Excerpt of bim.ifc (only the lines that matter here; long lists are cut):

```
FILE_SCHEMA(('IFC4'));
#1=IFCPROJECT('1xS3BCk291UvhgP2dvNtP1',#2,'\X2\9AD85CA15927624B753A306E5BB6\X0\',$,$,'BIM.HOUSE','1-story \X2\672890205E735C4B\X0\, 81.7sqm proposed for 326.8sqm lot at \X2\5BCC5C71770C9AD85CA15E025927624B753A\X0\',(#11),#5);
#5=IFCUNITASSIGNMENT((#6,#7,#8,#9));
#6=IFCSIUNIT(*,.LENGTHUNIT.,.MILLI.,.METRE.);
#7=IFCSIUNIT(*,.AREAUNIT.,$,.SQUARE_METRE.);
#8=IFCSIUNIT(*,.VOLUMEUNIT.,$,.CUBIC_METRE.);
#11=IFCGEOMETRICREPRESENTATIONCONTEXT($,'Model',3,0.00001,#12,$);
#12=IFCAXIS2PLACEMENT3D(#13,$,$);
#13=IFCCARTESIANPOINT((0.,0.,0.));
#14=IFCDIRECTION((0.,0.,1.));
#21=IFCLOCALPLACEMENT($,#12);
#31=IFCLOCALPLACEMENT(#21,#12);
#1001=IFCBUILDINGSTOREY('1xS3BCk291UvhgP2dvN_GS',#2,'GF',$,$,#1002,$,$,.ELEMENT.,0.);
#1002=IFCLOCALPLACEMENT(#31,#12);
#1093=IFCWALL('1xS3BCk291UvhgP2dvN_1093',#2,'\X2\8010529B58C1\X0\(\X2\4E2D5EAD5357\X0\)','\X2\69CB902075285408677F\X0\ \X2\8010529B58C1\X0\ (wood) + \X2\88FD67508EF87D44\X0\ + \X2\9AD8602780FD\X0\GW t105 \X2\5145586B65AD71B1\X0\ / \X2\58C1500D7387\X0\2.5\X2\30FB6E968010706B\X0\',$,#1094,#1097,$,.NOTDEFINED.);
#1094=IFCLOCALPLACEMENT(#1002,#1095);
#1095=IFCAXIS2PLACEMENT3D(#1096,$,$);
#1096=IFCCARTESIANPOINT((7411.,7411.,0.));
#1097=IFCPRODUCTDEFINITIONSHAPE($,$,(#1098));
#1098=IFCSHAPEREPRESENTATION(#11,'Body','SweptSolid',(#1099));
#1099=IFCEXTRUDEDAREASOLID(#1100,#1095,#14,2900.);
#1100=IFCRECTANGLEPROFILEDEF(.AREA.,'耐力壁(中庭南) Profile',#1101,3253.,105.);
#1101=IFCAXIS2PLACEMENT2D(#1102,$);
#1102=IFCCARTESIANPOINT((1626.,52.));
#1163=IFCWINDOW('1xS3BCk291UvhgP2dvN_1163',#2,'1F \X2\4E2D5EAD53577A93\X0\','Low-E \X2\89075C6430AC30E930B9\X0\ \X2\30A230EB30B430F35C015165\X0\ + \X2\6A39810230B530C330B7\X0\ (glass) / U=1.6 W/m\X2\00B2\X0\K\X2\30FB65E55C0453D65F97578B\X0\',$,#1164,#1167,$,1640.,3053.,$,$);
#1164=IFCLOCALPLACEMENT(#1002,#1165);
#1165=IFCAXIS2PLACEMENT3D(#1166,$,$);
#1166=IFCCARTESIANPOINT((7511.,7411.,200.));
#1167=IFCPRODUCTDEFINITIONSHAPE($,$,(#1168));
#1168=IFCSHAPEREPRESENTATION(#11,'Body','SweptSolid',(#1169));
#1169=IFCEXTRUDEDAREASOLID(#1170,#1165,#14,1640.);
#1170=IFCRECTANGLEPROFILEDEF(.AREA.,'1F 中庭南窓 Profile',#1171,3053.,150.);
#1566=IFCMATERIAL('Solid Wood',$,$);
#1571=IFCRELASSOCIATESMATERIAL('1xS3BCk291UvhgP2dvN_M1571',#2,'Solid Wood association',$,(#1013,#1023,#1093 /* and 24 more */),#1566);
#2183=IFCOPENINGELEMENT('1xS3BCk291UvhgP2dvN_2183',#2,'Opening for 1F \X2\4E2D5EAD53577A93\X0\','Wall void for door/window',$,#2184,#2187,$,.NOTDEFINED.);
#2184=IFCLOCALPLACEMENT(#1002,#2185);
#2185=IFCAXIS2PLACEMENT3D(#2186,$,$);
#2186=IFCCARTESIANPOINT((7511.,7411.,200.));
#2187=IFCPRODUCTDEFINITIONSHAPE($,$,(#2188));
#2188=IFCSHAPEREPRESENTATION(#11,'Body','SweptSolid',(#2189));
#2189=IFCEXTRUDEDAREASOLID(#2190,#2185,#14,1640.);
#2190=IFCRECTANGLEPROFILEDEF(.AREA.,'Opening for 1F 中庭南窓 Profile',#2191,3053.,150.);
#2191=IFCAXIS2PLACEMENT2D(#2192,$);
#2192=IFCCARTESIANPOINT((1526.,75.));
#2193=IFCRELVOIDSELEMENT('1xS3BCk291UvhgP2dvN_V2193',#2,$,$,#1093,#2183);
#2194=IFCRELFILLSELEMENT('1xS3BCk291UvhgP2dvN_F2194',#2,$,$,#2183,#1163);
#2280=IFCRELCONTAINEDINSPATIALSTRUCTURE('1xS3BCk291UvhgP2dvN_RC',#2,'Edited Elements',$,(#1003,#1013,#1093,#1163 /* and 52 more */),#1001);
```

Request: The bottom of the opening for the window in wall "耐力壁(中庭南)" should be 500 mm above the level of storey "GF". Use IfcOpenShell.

```python
import numpy as np
import ifcopenshell
import ifcopenshell.api.geometry
import ifcopenshell.geom
import ifcopenshell.util.element
import ifcopenshell.util.placement
import ifcopenshell.util.shape
import ifcopenshell.util.unit

model = ifcopenshell.open("bim.ifc")
unit_scale = ifcopenshell.util.unit.calculate_unit_scale(model)

window = model.by_guid("1xS3BCk291UvhgP2dvN_1163")
opening = window.FillsVoids[0].RelatingOpeningElement
storey = ifcopenshell.util.element.get_container(window, ifc_class="IfcBuildingStorey")
level = ifcopenshell.util.placement.get_local_placement(storey.ObjectPlacement)[2, 3]

# The opening's origin need not be at the sill, so measure its lowest point.
shape = ifcopenshell.geom.create_shape(ifcopenshell.geom.settings(), opening)
bottom = ifcopenshell.util.shape.get_shape_bottom_elevation(shape, shape.geometry) / unit_scale
dz = level + 0.5 / unit_scale - bottom

shift = np.array([0.0, 0.0, dz])
# The window is not placed relative to its opening, so move both.
for product in (opening, window):
    matrix = ifcopenshell.util.placement.get_local_placement(product.ObjectPlacement)
    matrix[:3, 3] += shift
    ifcopenshell.api.geometry.edit_object_placement(model, product=product, matrix=matrix, is_si=False)

print(f"moved by {dz * unit_scale:+.3f} m")

model.write("bim_edited.ifc")
```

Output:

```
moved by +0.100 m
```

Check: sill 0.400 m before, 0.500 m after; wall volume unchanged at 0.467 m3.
